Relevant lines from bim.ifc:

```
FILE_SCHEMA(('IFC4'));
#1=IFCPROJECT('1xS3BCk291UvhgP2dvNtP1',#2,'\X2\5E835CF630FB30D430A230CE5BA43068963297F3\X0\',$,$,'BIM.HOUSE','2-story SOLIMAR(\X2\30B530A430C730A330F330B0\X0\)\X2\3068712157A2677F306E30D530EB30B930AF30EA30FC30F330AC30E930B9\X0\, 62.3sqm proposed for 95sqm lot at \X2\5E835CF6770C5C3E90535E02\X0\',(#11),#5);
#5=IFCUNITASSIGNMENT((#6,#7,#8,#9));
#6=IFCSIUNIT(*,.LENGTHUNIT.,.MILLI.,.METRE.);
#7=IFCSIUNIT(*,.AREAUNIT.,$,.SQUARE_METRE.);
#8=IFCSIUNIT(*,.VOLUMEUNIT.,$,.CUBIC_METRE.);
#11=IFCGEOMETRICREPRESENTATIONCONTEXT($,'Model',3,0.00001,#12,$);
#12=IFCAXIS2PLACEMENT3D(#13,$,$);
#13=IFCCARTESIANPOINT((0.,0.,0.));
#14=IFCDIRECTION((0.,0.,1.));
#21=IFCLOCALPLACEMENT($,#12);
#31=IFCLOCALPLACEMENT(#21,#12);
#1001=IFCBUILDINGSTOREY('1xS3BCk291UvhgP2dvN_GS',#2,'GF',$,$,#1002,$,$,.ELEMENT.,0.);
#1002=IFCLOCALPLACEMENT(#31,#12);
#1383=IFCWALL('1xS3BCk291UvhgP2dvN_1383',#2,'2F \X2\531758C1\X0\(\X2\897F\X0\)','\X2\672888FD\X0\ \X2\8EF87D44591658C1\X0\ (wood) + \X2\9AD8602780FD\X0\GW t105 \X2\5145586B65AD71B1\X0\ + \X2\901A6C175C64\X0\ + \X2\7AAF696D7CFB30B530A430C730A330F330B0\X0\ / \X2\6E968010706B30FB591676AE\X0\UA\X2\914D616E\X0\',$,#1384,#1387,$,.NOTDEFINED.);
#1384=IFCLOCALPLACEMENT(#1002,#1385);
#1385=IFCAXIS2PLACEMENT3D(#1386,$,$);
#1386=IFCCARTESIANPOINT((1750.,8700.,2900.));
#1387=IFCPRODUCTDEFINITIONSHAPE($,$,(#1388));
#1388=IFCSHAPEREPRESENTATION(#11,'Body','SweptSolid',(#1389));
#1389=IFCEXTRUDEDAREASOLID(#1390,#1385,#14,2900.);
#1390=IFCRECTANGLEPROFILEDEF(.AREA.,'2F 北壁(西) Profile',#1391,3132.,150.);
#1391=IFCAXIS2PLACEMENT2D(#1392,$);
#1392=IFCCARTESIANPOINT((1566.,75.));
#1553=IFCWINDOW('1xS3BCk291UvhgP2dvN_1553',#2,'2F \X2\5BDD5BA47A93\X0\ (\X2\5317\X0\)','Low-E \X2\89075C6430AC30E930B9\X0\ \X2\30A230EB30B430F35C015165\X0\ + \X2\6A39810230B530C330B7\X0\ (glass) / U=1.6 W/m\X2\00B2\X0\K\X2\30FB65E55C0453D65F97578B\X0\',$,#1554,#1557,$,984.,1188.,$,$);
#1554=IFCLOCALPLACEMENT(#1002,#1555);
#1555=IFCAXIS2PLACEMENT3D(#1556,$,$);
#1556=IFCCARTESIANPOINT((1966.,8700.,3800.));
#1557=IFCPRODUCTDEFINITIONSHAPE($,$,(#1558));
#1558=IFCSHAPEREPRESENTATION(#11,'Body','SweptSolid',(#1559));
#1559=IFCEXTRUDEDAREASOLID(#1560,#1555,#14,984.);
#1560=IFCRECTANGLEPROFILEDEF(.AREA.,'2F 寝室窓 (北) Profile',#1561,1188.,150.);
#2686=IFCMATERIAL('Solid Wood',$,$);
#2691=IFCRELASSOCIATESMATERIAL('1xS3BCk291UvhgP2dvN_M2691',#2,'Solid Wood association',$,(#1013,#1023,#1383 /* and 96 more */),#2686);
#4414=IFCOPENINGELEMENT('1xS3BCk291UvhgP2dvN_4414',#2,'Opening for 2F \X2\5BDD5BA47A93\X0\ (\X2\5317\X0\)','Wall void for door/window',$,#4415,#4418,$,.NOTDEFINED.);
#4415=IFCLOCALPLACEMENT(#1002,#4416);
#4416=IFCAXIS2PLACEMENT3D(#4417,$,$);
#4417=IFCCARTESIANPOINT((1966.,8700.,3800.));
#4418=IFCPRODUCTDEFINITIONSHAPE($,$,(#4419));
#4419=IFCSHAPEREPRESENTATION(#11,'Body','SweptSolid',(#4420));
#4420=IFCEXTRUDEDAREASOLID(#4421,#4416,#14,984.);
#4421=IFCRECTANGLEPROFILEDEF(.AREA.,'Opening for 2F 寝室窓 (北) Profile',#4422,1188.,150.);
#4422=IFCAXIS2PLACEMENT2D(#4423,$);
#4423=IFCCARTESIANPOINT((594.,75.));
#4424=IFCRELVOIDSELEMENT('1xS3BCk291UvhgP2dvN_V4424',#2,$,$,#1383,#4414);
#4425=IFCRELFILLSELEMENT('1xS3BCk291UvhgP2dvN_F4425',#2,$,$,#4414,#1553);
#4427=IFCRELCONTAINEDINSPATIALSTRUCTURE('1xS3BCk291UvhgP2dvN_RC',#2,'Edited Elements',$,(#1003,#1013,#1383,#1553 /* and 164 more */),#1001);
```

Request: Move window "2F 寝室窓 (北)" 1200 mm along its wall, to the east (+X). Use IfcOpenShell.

```python
import ifcopenshell
import ifcopenshell.api.geometry
import ifcopenshell.util.placement
import ifcopenshell.util.unit

model = ifcopenshell.open("bim.ifc")
unit_scale = ifcopenshell.util.unit.calculate_unit_scale(model)

window = model.by_guid("1xS3BCk291UvhgP2dvN_1553")
opening = window.FillsVoids[0].RelatingOpeningElement
wall = opening.VoidsElements[0].RelatingBuildingElement

wall_matrix = ifcopenshell.util.placement.get_local_placement(wall.ObjectPlacement)
shift = wall_matrix[:3, 0] * 1.2 / unit_scale
before = ifcopenshell.util.placement.get_local_placement(window.ObjectPlacement)[:3, 3].copy()

# The window is not placed relative to its opening, so move both.
for product in (opening, window):
    matrix = ifcopenshell.util.placement.get_local_placement(product.ObjectPlacement)
    matrix[:3, 3] += shift
    ifcopenshell.api.geometry.edit_object_placement(model, product=product, matrix=matrix, is_si=False)

after = ifcopenshell.util.placement.get_local_placement(window.ObjectPlacement)[:3, 3]
print("window moved by", (after - before).round(3) + 0.0)

model.write("bim_edited.ifc")
```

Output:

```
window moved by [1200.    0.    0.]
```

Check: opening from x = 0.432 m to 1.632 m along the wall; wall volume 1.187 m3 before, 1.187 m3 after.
